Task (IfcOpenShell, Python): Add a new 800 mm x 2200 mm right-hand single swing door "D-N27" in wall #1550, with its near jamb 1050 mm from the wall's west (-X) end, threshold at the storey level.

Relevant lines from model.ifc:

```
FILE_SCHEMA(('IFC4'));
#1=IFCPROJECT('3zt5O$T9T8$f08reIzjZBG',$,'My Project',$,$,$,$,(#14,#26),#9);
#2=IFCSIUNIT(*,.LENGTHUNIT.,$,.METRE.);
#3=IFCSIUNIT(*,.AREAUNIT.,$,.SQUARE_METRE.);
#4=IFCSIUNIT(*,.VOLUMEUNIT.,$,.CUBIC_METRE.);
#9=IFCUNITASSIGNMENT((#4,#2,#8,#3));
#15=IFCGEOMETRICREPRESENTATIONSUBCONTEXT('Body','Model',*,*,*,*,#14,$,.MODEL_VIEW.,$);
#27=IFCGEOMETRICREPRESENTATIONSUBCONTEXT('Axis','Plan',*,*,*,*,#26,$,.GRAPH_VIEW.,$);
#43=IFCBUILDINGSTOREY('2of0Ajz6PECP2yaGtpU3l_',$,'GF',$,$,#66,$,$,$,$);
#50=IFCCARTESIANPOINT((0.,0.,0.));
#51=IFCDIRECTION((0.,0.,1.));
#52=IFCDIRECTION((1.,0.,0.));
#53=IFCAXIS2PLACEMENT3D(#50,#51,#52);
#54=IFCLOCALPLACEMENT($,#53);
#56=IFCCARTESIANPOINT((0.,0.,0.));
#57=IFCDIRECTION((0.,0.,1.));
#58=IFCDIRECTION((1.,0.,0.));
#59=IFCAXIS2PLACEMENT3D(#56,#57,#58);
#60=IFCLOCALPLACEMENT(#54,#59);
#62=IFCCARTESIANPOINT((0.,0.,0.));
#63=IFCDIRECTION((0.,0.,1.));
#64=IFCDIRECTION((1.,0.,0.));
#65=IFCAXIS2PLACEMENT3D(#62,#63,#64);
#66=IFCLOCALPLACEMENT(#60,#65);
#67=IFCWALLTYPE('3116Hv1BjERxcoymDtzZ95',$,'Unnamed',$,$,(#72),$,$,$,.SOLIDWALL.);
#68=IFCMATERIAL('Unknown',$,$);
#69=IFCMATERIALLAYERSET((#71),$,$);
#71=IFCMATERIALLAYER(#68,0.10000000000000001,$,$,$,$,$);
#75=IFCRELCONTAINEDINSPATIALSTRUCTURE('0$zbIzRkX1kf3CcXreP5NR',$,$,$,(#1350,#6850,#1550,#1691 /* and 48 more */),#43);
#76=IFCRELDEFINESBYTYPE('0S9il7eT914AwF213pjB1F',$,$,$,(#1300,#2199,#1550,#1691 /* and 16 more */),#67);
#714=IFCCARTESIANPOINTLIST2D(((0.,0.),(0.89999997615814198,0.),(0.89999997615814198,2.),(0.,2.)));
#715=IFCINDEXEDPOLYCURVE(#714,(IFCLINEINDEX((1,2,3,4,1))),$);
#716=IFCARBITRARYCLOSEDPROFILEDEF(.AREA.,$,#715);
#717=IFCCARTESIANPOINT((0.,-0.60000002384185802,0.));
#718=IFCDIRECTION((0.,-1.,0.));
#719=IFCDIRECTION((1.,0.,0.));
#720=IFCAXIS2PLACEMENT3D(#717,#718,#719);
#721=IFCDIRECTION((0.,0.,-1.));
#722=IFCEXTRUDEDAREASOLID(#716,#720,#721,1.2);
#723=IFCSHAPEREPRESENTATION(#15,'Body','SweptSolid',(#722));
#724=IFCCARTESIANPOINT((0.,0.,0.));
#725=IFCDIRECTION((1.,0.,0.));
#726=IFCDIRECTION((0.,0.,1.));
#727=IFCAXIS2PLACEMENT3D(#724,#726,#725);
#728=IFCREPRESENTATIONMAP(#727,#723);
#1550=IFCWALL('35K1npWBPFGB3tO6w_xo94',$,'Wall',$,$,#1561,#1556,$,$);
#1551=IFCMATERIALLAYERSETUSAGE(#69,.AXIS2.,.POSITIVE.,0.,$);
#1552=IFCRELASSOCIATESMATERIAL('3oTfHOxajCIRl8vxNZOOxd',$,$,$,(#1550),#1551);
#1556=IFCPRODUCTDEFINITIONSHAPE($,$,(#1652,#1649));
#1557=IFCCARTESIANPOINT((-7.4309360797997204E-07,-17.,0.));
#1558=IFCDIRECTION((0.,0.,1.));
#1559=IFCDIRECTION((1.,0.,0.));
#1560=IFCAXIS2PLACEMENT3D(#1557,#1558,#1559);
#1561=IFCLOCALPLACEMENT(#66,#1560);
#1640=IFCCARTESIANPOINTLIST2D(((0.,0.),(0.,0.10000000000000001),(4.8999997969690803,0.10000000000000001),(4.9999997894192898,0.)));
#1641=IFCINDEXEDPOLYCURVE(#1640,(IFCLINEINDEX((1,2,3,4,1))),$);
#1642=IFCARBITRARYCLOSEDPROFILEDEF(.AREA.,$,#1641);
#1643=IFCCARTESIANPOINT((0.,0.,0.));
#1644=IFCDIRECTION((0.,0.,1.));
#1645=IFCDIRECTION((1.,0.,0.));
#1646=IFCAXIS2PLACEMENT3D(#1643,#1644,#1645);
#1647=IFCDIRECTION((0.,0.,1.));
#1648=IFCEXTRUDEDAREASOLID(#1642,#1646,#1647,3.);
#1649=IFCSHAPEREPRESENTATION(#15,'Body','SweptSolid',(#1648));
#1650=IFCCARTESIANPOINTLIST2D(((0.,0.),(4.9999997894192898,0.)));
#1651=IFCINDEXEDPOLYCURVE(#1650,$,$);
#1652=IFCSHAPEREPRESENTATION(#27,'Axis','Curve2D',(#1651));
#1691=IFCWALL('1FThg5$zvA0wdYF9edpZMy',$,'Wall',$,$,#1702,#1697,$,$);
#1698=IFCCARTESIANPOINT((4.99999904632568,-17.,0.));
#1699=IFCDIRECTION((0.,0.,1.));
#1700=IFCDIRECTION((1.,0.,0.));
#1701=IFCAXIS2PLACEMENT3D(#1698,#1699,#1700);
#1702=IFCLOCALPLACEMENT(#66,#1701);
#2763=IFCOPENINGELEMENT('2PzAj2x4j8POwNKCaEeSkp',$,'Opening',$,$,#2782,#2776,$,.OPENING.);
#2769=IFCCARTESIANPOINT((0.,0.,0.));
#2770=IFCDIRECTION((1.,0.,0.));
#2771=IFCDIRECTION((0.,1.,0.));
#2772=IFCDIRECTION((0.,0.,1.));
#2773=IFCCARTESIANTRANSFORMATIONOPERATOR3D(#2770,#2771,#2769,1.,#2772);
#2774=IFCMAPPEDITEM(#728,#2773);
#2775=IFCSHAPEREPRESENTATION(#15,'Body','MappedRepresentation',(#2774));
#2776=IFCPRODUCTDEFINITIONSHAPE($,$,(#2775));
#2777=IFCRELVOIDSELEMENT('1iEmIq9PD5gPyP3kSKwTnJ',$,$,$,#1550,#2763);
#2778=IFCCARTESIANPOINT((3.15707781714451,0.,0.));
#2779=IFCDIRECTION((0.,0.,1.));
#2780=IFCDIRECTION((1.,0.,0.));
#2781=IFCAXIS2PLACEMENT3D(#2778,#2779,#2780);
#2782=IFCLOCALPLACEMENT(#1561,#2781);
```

```python
import numpy as np
import ifcopenshell
import ifcopenshell.api.feature
import ifcopenshell.api.geometry
import ifcopenshell.api.root
import ifcopenshell.api.spatial
import ifcopenshell.geom
import ifcopenshell.util.element
import ifcopenshell.util.placement
import ifcopenshell.util.representation
import ifcopenshell.util.shape
import ifcopenshell.util.unit

model = ifcopenshell.open("model.ifc")
unit_scale = ifcopenshell.util.unit.calculate_unit_scale(model)
settings = ifcopenshell.geom.settings()


def volume(element):
    """Net volume in cubic metres, openings subtracted."""
    shape = ifcopenshell.geom.create_shape(settings, element)
    return ifcopenshell.util.shape.get_volume(shape.geometry)


wall = model.by_id(1550)
storey = ifcopenshell.util.element.get_container(wall, ifc_class="IfcBuildingStorey")
context = ifcopenshell.util.representation.get_context(model, "Model", "Body", "MODEL_VIEW")
before = volume(wall)

width, height, from_end, sill = 0.8, 2.2, 1.05, 0.0  # metres

# The wall runs along its own X axis, and the end named is its -X end.
wall_shape = ifcopenshell.geom.create_shape(settings, wall)
x, y, z = ifcopenshell.util.shape.get_vertices(wall_shape.geometry).T
start = x.min() + from_end
face, thickness = float(y.min()), float(y.max() - y.min())
wall_matrix = ifcopenshell.util.placement.get_local_placement(wall.ObjectPlacement)
level = ifcopenshell.util.placement.get_local_placement(storey.ObjectPlacement)[2, 3]


def in_wall(x, y):
    """Placement at x, y metres in the wall's axes, at sill height."""
    matrix = wall_matrix.copy()
    matrix[:, 3] = wall_matrix @ np.array([x / unit_scale, y / unit_scale, 0.0, 1.0])
    matrix[2, 3] = level + sill / unit_scale
    return matrix


# Opening: a box that overshoots both wall faces by 50 mm.
opening = ifcopenshell.api.root.create_entity(model, ifc_class="IfcOpeningElement", predefined_type="OPENING")
box = ifcopenshell.api.geometry.add_wall_representation(
    model, context=context, length=width, height=height, thickness=thickness + 0.1
)
ifcopenshell.api.geometry.assign_representation(model, product=opening, representation=box)
ifcopenshell.api.geometry.edit_object_placement(model, product=opening, matrix=in_wall(start, face - 0.05), is_si=False)
ifcopenshell.api.feature.add_feature(model, feature=opening, element=wall)

door = ifcopenshell.api.root.create_entity(model, ifc_class="IfcDoor", name="D-N27", predefined_type="DOOR")
door.OverallWidth, door.OverallHeight = width / unit_scale, height / unit_scale
door.OperationType = "SINGLE_SWING_RIGHT"
body = ifcopenshell.api.geometry.add_door_representation(
    model,
    context=context,
    overall_width=door.OverallWidth,
    overall_height=door.OverallHeight,
    operation_type="SINGLE_SWING_RIGHT",
    lining_properties={"LiningDepth": thickness / unit_scale, "ThresholdDepth": thickness / unit_scale},
)
ifcopenshell.api.geometry.assign_representation(model, product=door, representation=body)
ifcopenshell.api.spatial.assign_container(model, products=[door], relating_structure=storey)
ifcopenshell.api.feature.add_filling(model, opening=opening, element=door)

# The lining spans the wall, so the door starts at the wall face.
ifcopenshell.api.geometry.edit_object_placement(model, product=door, matrix=in_wall(start, face), is_si=False)

after = volume(wall)

print(f"wall volume {before:.3f} -> {after:.3f} m3")

model.write("model_v2.ifc")
```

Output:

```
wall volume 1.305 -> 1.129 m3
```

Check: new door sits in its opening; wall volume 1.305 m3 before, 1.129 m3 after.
